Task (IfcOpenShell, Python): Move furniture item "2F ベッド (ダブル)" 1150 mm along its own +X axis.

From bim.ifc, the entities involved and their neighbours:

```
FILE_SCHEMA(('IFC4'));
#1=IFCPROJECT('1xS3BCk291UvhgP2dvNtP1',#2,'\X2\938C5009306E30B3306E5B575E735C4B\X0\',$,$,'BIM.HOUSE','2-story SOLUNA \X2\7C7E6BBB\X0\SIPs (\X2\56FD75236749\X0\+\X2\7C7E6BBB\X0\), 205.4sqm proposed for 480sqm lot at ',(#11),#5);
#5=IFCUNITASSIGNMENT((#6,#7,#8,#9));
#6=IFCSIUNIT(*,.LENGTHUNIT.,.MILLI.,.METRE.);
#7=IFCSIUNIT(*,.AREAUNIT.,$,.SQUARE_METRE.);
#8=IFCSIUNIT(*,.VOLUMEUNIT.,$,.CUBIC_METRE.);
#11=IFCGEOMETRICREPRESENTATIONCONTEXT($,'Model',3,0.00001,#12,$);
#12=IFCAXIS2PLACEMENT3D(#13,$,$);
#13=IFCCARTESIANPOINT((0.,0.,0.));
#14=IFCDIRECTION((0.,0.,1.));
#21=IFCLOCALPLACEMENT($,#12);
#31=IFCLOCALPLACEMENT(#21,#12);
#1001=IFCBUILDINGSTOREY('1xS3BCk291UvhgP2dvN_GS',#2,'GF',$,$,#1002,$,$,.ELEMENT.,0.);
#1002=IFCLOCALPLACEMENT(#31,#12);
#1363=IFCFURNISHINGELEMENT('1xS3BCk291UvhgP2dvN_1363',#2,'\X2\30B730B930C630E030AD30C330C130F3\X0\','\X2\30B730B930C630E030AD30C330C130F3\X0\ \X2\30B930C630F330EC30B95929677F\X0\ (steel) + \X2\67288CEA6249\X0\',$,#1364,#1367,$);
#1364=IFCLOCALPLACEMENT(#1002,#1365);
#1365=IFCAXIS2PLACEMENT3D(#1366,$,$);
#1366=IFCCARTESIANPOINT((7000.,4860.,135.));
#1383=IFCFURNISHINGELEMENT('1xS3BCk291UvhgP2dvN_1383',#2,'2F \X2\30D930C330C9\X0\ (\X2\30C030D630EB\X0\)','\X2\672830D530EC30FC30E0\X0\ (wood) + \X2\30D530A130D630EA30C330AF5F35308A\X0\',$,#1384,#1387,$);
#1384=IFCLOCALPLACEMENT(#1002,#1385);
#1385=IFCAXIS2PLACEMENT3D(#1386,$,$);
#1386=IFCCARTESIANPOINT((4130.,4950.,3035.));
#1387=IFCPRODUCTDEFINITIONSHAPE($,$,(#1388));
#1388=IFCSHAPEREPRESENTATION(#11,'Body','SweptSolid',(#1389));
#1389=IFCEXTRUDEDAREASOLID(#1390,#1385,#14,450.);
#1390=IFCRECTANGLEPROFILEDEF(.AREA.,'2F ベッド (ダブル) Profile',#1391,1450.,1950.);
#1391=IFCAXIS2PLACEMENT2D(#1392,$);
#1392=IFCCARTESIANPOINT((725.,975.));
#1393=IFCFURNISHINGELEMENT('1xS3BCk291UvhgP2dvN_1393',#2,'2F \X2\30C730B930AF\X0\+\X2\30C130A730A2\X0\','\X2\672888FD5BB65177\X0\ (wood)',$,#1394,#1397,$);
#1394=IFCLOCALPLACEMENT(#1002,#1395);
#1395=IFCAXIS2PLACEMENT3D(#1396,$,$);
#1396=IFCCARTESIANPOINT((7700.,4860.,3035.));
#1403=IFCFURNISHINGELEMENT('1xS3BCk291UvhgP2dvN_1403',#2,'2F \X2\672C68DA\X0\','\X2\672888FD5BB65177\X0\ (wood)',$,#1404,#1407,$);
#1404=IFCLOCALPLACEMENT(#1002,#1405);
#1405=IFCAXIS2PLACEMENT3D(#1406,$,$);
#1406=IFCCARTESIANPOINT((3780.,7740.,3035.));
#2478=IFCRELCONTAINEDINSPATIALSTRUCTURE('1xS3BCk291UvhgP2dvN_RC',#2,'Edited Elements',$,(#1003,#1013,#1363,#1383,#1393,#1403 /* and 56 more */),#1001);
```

```python
import ifcopenshell
import ifcopenshell.api.geometry
import ifcopenshell.util.placement

model = ifcopenshell.open("bim.ifc")

item = model.by_guid("1xS3BCk291UvhgP2dvN_1383")
matrix = ifcopenshell.util.placement.get_local_placement(item.ObjectPlacement)
matrix[:3, 3] += matrix[:3, 0] * 1150.0
ifcopenshell.api.geometry.edit_object_placement(model, product=item, matrix=matrix, is_si=False)

print(ifcopenshell.util.placement.get_local_placement(item.ObjectPlacement).round(3) + 0.0)

model.write("bim_updated.ifc")
```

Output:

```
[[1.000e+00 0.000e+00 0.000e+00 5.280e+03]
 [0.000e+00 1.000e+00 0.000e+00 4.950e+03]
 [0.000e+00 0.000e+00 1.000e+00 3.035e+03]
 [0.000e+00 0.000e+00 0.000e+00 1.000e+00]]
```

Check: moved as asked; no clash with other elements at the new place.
